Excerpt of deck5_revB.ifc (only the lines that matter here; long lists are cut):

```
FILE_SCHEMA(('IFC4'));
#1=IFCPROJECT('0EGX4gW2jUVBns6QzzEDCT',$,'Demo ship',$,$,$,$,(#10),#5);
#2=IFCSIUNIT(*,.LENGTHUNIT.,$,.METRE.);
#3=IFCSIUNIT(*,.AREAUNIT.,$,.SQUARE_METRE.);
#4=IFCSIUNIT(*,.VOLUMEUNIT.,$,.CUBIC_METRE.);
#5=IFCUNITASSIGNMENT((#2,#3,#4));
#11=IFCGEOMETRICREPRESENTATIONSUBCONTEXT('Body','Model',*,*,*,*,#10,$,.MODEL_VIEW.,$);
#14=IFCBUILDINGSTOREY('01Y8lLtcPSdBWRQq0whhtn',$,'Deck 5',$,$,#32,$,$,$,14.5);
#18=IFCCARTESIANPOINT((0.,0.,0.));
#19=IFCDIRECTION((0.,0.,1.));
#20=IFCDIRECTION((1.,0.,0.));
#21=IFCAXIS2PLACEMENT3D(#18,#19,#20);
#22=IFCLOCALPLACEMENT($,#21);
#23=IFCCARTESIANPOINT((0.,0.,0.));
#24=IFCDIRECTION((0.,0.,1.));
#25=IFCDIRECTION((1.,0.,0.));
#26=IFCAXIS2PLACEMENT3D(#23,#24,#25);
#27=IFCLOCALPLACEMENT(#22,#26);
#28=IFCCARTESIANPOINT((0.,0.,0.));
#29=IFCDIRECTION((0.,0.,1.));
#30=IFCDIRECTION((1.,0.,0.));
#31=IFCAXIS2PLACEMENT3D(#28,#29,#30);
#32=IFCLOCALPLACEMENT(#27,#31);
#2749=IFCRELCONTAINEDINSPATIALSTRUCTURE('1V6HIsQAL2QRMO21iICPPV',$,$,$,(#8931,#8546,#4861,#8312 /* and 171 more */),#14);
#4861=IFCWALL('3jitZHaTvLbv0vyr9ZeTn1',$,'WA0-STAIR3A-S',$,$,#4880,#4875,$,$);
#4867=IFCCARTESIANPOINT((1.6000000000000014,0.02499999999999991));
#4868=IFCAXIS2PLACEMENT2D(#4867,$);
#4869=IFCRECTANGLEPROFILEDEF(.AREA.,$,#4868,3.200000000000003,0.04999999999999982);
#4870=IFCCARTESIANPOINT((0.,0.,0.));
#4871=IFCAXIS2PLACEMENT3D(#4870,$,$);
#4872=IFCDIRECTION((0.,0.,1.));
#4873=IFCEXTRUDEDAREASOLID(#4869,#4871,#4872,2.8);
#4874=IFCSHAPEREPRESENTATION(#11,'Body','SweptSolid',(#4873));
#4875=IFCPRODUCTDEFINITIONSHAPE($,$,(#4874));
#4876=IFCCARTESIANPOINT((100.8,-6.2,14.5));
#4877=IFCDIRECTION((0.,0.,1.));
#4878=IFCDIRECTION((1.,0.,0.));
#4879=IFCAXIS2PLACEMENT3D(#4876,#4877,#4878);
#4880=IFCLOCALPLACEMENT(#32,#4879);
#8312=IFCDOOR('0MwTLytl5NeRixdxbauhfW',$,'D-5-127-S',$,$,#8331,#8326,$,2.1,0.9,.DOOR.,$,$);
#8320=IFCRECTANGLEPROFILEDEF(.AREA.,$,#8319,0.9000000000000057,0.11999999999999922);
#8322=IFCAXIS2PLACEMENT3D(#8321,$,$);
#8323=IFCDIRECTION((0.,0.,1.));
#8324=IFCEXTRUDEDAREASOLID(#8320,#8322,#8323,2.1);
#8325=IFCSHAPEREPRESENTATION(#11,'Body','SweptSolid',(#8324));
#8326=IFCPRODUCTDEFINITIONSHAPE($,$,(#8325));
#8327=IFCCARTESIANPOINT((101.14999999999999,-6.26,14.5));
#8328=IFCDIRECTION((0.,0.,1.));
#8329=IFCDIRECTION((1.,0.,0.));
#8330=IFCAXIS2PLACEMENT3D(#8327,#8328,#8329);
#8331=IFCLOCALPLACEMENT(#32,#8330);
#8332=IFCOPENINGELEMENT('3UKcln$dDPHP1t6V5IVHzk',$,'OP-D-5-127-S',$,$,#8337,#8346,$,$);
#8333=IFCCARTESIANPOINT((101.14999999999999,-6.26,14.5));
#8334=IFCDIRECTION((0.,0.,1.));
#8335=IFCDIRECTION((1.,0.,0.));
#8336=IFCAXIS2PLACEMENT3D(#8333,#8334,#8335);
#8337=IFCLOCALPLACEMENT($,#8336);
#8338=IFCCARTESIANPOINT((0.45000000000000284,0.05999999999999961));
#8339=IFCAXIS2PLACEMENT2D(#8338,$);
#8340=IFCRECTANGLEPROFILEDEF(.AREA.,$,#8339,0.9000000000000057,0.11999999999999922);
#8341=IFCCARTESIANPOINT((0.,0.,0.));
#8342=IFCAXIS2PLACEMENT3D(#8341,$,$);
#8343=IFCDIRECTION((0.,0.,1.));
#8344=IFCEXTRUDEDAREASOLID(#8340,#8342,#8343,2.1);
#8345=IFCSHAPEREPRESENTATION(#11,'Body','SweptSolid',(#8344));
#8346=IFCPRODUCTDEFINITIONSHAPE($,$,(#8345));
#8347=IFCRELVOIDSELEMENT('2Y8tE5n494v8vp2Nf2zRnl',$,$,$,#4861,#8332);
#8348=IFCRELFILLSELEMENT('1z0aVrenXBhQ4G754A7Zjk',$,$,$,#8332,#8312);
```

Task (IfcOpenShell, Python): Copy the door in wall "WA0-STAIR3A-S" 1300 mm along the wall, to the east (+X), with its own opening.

```python
import ifcopenshell
import ifcopenshell.api.feature
import ifcopenshell.api.geometry
import ifcopenshell.api.root
import ifcopenshell.geom
import ifcopenshell.util.element
import ifcopenshell.util.placement
import ifcopenshell.util.shape

model = ifcopenshell.open("deck5_revB.ifc")
settings = ifcopenshell.geom.settings()


def volume(element):
    """Net volume in cubic metres, openings subtracted."""
    shape = ifcopenshell.geom.create_shape(settings, element)
    return ifcopenshell.util.shape.get_volume(shape.geometry)


door = model.by_guid("0MwTLytl5NeRixdxbauhfW")
opening = door.FillsVoids[0].RelatingOpeningElement
wall = opening.VoidsElements[0].RelatingBuildingElement
before = volume(wall)
shift = ifcopenshell.util.placement.get_local_placement(wall.ObjectPlacement)[:3, 0] * 1.3

# copy_class copies the void relationship, type, container and properties, but no geometry.
new_opening = ifcopenshell.api.root.copy_class(model, product=opening)
new_opening.Representation = ifcopenshell.util.element.copy_deep(
    model, opening.Representation, exclude=["IfcGeometricRepresentationContext", "IfcRepresentationMap"]
)
new_door = ifcopenshell.api.root.copy_class(model, product=door)
new_door.Representation = ifcopenshell.util.element.copy_deep(
    model, door.Representation, exclude=["IfcGeometricRepresentationContext", "IfcRepresentationMap"]
)
ifcopenshell.api.feature.add_filling(model, opening=new_opening, element=new_door)

for old, new in ((opening, new_opening), (door, new_door)):
    matrix = ifcopenshell.util.placement.get_local_placement(old.ObjectPlacement)
    matrix[:3, 3] += shift
    ifcopenshell.api.geometry.edit_object_placement(model, product=new, matrix=matrix, is_si=False)

after = volume(wall)

print(f"wall volume {before:.3f} -> {after:.3f} m3")

model.write("deck5_revB_v2.ifc")
```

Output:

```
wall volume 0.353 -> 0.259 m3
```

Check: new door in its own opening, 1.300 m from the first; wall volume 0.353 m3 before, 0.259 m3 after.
